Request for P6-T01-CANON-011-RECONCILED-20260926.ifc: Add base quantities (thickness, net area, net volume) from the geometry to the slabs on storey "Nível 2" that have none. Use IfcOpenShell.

First a look at what the model holds.

```python
import ifcopenshell
import ifcopenshell.util.element
import ifcopenshell.util.unit

model = ifcopenshell.open("P6-T01-CANON-011-RECONCILED-20260926.ifc")
print(model.schema)
for unit_type in ("LENGTHUNIT", "AREAUNIT", "VOLUMEUNIT"):
    print(unit_type, ifcopenshell.util.unit.calculate_unit_scale(model, unit_type))
storey = next(s for s in model.by_type("IfcBuildingStorey") if s.Name == "Nível 2")
slabs = [e for e in ifcopenshell.util.element.get_decomposition(storey) if e.is_a("IfcSlab")]
for e in sorted(slabs, key=lambda e: e.id()):
    print(e.id(), e.is_a(), e.Name, list(ifcopenshell.util.element.get_psets(e, qtos_only=True)), sep=" | ")
```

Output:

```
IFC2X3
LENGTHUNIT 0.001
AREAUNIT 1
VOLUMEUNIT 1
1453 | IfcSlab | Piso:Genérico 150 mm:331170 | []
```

```python
import ifcopenshell
import ifcopenshell.api.pset
import ifcopenshell.geom
import ifcopenshell.util.element
import ifcopenshell.util.shape
import ifcopenshell.util.unit

model = ifcopenshell.open("P6-T01-CANON-011-RECONCILED-20260926.ifc")
unit_scale = ifcopenshell.util.unit.calculate_unit_scale(model)
area_scale = ifcopenshell.util.unit.calculate_unit_scale(model, "AREAUNIT")
volume_scale = ifcopenshell.util.unit.calculate_unit_scale(model, "VOLUMEUNIT")
settings = ifcopenshell.geom.settings()

storey = next(s for s in model.by_type("IfcBuildingStorey") if s.Name == "Nível 2")
slabs = [e for e in ifcopenshell.util.element.get_decomposition(storey) if e.is_a("IfcSlab")]

for e in sorted(slabs, key=lambda e: e.id()):
    if ifcopenshell.util.element.get_psets(e, qtos_only=True, should_inherit=False):
        continue
    # Geometry comes back in metres, in the element's own axes.
    shape = ifcopenshell.geom.create_shape(settings, e)
    values = {
        "Width": ifcopenshell.util.shape.get_z(shape.geometry) / unit_scale,
        "NetArea": ifcopenshell.util.shape.get_footprint_area(shape.geometry) / area_scale,
        "NetVolume": ifcopenshell.util.shape.get_volume(shape.geometry) / volume_scale,
    }
    qto = ifcopenshell.api.pset.add_qto(model, product=e, name="BaseQuantities")
    ifcopenshell.api.pset.edit_qto(model, qto=qto, properties=values)
    print(e.id(), {k: round(v, 3) for k, v in values.items()})

model.write("P6-T01-CANON-011-RECONCILED-20260926_rev.ifc")
```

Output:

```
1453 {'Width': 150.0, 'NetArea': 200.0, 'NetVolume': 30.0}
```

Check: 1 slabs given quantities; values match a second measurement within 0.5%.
